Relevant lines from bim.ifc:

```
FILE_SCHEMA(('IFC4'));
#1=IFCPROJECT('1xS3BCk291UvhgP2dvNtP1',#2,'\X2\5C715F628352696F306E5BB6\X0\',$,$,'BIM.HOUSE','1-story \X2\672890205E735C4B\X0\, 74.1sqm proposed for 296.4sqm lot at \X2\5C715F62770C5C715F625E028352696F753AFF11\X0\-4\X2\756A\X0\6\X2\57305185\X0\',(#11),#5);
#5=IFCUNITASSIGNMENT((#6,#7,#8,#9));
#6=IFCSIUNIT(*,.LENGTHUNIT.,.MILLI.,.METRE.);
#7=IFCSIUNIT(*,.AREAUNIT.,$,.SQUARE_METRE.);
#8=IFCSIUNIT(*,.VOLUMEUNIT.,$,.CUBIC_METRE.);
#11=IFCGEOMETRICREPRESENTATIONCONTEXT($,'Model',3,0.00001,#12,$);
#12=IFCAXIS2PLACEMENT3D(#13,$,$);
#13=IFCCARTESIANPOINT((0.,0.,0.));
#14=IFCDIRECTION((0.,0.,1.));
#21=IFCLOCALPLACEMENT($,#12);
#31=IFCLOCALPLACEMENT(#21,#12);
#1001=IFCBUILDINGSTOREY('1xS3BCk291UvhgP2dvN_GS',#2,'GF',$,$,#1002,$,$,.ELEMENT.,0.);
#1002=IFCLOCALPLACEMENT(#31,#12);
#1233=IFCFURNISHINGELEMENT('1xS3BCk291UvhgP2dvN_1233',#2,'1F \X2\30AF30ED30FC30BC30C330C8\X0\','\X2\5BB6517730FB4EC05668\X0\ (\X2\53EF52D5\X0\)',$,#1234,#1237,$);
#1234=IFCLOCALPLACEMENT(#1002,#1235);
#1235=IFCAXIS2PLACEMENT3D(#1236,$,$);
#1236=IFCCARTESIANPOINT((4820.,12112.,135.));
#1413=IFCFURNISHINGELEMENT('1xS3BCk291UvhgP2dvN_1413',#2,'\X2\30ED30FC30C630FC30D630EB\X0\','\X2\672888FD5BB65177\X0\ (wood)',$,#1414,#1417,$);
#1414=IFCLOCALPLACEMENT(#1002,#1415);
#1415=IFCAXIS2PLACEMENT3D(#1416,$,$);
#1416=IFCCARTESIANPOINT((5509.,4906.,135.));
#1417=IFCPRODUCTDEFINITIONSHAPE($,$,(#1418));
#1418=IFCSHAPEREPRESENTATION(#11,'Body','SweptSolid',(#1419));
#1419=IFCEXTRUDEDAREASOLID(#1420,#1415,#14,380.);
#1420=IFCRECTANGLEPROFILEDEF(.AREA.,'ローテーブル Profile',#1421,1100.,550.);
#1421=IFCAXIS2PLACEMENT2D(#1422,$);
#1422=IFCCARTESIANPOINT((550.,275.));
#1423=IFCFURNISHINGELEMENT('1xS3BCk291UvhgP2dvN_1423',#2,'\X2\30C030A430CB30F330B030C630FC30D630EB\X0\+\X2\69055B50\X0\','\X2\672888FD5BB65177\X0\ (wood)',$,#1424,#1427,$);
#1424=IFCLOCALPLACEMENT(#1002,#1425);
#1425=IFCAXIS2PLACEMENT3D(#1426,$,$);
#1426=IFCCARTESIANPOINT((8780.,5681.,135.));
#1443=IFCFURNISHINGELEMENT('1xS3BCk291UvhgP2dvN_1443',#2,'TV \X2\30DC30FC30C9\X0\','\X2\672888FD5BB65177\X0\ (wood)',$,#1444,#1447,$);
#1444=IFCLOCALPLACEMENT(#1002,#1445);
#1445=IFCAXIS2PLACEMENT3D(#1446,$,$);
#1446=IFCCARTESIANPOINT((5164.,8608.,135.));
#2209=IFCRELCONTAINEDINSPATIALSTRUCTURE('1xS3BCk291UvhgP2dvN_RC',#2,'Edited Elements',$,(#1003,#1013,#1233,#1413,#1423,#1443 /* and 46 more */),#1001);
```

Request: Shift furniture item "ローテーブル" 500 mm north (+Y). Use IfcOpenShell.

```python
import ifcopenshell
import ifcopenshell.api.geometry
import ifcopenshell.util.placement
import ifcopenshell.util.unit

model = ifcopenshell.open("bim.ifc")
unit_scale = ifcopenshell.util.unit.calculate_unit_scale(model)

item = model.by_id(1413)
matrix = ifcopenshell.util.placement.get_local_placement(item.ObjectPlacement)
matrix[1, 3] += 0.5 / unit_scale
ifcopenshell.api.geometry.edit_object_placement(model, product=item, matrix=matrix, is_si=False)

print(ifcopenshell.util.placement.get_local_placement(item.ObjectPlacement).round(3) + 0.0)

model.write("bim-out.ifc")
```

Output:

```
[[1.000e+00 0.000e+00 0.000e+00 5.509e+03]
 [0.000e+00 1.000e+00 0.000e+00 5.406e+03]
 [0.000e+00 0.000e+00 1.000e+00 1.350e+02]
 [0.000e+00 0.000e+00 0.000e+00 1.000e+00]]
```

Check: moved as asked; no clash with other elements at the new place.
